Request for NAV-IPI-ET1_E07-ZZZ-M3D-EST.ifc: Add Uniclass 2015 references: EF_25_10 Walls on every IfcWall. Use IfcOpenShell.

First a look at what the model holds.

```python
import ifcopenshell

model = ifcopenshell.open("NAV-IPI-ET1_E07-ZZZ-M3D-EST.ifc")
print(model.schema)
print("classifications:", [c.Name for c in model.by_type("IfcClassification")])
for ifc_class in ("IfcDoor", "IfcRoof", "IfcStair", "IfcWall", "IfcWindow"):
    print(ifc_class, len(model.by_type(ifc_class)))
```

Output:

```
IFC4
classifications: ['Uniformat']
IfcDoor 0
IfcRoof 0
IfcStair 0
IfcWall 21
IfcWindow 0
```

```python
import ifcopenshell
import ifcopenshell.api.classification

model = ifcopenshell.open("NAV-IPI-ET1_E07-ZZZ-M3D-EST.ifc")

system = ifcopenshell.api.classification.add_classification(model, classification="Uniclass 2015")

codes = {
    "IfcWall": ("EF_25_10", "Walls"),
}
for ifc_class, (code, name) in codes.items():
    products = model.by_type(ifc_class)
    ifcopenshell.api.classification.add_reference(
        model, products=products, classification=system, identification=code, name=name
    )
    print(code, len(products))

model.write("NAV-IPI-ET1_E07-ZZZ-M3D-EST_edited.ifc")
```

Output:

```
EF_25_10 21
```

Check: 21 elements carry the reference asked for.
